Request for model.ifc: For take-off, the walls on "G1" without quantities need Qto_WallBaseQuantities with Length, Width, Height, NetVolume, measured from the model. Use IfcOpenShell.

First a look at what the model holds.

```python
import ifcopenshell
import ifcopenshell.util.element
import ifcopenshell.util.unit

model = ifcopenshell.open("model.ifc")
print(model.schema)
for unit_type in ("LENGTHUNIT", "AREAUNIT", "VOLUMEUNIT"):
    print(unit_type, ifcopenshell.util.unit.calculate_unit_scale(model, unit_type))
storey = next(s for s in model.by_type("IfcBuildingStorey") if s.Name == "G1")
walls = [e for e in ifcopenshell.util.element.get_decomposition(storey) if e.is_a("IfcWall")]
for e in sorted(walls, key=lambda e: e.id()):
    print(e.id(), e.is_a(), e.Name, list(ifcopenshell.util.element.get_psets(e, qtos_only=True)), sep=" | ")
```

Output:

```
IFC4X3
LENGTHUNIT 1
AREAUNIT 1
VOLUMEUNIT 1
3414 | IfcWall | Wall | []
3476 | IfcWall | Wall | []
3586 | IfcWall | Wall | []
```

```python
import ifcopenshell
import ifcopenshell.api.pset
import ifcopenshell.geom
import ifcopenshell.util.element
import ifcopenshell.util.shape
import ifcopenshell.util.unit

model = ifcopenshell.open("model.ifc")
unit_scale = ifcopenshell.util.unit.calculate_unit_scale(model)
volume_scale = ifcopenshell.util.unit.calculate_unit_scale(model, "VOLUMEUNIT")
settings = ifcopenshell.geom.settings()

storey = next(s for s in model.by_type("IfcBuildingStorey") if s.Name == "G1")
walls = [e for e in ifcopenshell.util.element.get_decomposition(storey) if e.is_a("IfcWall")]

for e in sorted(walls, key=lambda e: e.id()):
    if ifcopenshell.util.element.get_psets(e, qtos_only=True, should_inherit=False):
        continue
    # Geometry comes back in metres, in the element's own axes.
    shape = ifcopenshell.geom.create_shape(settings, e)
    values = {
        "Length": ifcopenshell.util.shape.get_x(shape.geometry) / unit_scale,
        "Width": ifcopenshell.util.shape.get_y(shape.geometry) / unit_scale,
        "Height": ifcopenshell.util.shape.get_z(shape.geometry) / unit_scale,
        "NetVolume": ifcopenshell.util.shape.get_volume(shape.geometry) / volume_scale,
    }
    qto = ifcopenshell.api.pset.add_qto(model, product=e, name="Qto_WallBaseQuantities")
    ifcopenshell.api.pset.edit_qto(model, qto=qto, properties=values)
    print(e.id(), {k: round(v, 3) for k, v in values.items()})

model.write("model_v2.ifc")
```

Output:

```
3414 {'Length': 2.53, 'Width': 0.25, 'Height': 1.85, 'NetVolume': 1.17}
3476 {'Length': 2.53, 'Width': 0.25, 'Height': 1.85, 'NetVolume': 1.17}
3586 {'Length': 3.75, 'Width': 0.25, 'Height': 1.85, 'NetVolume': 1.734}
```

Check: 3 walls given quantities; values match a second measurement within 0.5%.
